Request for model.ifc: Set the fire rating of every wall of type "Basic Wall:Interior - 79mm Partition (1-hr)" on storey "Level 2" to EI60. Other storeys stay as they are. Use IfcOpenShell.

First a look at what the model holds.

```python
import ifcopenshell
import ifcopenshell.util.element

model = ifcopenshell.open("model.ifc")
print(model.schema)
storey = next(s for s in model.by_type("IfcBuildingStorey") if s.Name == "Level 2")
walls = [e for e in ifcopenshell.util.element.get_decomposition(storey) if e.is_a("IfcWall")]
seen = {}
for e in walls:
    element_type = ifcopenshell.util.element.get_type(e)
    key = (element_type.Name if element_type != e and element_type else None, ifcopenshell.util.element.get_pset(e, "Pset_WallCommon", "FireRating"))
    seen[key] = seen.get(key, 0) + 1
for (name, value), count in sorted(seen.items(), key=str):
    print(count, "x", name, "|", value)
```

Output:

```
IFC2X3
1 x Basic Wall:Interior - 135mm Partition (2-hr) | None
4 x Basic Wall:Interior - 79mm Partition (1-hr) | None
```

```python
import ifcopenshell
import ifcopenshell.api.pset
import ifcopenshell.util.element

model = ifcopenshell.open("model.ifc")

storey = next(s for s in model.by_type("IfcBuildingStorey") if s.Name == "Level 2")
walls = [e for e in ifcopenshell.util.element.get_decomposition(storey) if e.is_a("IfcWall")]

count = 0
for e in walls:
    element_type = ifcopenshell.util.element.get_type(e)
    if element_type in (None, e) or element_type.Name != "Basic Wall:Interior - 79mm Partition (1-hr)":
        continue
    # add_pset returns the element's existing set when there is one.
    pset = ifcopenshell.api.pset.add_pset(model, product=e, name="Pset_WallCommon")
    ifcopenshell.api.pset.edit_pset(model, pset=pset, properties={"FireRating": "EI60"})
    count += 1

print(count, "walls updated")

model.write("model_v2.ifc")
```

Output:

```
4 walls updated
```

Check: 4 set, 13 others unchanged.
